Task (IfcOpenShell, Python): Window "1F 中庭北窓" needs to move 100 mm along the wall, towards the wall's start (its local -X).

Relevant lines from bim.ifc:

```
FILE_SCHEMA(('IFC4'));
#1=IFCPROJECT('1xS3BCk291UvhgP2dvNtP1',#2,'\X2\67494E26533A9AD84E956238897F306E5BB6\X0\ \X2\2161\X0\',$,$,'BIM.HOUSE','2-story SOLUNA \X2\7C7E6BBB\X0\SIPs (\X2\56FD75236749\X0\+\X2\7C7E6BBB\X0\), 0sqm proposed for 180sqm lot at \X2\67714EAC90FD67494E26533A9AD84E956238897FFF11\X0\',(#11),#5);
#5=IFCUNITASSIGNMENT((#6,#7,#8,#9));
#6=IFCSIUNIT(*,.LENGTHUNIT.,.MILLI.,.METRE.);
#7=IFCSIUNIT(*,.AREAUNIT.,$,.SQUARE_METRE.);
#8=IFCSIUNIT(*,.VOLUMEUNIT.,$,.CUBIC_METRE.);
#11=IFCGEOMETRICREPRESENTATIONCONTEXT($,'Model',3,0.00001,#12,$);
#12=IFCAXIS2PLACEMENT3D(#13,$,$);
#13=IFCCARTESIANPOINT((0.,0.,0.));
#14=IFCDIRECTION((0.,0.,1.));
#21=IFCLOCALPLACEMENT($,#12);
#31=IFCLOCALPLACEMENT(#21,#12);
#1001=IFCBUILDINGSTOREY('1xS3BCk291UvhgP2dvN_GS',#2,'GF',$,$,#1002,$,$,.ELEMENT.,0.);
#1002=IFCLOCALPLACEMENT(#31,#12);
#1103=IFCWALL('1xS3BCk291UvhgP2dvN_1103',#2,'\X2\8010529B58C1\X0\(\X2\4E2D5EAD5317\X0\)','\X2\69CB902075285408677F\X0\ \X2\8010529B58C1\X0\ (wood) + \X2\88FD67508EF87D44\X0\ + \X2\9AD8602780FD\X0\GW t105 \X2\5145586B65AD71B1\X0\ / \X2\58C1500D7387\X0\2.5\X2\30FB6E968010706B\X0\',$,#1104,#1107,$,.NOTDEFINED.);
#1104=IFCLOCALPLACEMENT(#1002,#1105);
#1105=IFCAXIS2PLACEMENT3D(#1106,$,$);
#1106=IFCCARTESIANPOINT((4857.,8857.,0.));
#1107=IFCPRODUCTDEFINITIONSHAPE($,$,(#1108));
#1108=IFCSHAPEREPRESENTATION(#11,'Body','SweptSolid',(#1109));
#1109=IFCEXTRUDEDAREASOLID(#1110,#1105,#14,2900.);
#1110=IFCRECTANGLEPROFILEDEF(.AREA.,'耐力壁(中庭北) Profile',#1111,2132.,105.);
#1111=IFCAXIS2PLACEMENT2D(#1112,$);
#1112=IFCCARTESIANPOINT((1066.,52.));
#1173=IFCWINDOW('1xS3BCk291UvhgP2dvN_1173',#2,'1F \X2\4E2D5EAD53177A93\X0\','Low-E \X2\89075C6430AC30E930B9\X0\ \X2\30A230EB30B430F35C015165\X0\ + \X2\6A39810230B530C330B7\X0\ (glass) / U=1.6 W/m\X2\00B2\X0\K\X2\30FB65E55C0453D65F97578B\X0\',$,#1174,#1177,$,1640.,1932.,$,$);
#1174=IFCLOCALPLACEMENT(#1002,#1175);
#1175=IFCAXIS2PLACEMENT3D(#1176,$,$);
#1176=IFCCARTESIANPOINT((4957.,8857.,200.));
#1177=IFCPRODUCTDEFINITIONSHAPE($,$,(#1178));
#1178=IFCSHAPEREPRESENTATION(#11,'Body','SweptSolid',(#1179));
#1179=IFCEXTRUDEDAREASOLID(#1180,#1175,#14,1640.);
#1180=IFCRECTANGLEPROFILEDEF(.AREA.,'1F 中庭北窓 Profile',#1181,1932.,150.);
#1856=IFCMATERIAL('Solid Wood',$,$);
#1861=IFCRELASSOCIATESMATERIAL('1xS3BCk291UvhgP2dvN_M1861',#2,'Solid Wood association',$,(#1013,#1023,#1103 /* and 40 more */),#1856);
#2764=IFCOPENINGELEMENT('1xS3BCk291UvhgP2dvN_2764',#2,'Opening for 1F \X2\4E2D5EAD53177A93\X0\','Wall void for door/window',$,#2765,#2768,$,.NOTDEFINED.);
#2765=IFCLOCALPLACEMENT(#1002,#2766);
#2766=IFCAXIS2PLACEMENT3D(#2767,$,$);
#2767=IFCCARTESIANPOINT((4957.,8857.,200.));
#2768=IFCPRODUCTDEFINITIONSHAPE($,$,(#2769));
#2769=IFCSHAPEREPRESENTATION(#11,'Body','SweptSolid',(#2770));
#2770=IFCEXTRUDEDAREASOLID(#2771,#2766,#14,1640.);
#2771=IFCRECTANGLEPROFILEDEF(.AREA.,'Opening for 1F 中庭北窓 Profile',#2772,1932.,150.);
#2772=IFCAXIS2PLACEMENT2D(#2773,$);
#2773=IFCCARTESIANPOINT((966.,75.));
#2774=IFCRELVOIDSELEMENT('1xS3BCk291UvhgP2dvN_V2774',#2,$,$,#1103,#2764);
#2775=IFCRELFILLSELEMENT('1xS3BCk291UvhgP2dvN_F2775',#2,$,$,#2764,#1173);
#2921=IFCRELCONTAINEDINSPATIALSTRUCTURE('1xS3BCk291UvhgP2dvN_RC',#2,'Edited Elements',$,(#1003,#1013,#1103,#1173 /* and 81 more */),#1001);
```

```python
import ifcopenshell
import ifcopenshell.api.geometry
import ifcopenshell.util.placement
import ifcopenshell.util.unit

model = ifcopenshell.open("bim.ifc")
unit_scale = ifcopenshell.util.unit.calculate_unit_scale(model)

window = model.by_guid("1xS3BCk291UvhgP2dvN_1173")
opening = window.FillsVoids[0].RelatingOpeningElement
wall = opening.VoidsElements[0].RelatingBuildingElement

wall_matrix = ifcopenshell.util.placement.get_local_placement(wall.ObjectPlacement)
shift = wall_matrix[:3, 0] * -0.1 / unit_scale
before = ifcopenshell.util.placement.get_local_placement(window.ObjectPlacement)[:3, 3].copy()

# The window is not placed relative to its opening, so move both.
for product in (opening, window):
    matrix = ifcopenshell.util.placement.get_local_placement(product.ObjectPlacement)
    matrix[:3, 3] += shift
    ifcopenshell.api.geometry.edit_object_placement(model, product=product, matrix=matrix, is_si=False)

after = ifcopenshell.util.placement.get_local_placement(window.ObjectPlacement)[:3, 3]
print("window moved by", (after - before).round(3) + 0.0)

model.write("bim_rev.ifc")
```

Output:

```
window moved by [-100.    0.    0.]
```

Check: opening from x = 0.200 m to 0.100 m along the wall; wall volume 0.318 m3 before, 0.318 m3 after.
